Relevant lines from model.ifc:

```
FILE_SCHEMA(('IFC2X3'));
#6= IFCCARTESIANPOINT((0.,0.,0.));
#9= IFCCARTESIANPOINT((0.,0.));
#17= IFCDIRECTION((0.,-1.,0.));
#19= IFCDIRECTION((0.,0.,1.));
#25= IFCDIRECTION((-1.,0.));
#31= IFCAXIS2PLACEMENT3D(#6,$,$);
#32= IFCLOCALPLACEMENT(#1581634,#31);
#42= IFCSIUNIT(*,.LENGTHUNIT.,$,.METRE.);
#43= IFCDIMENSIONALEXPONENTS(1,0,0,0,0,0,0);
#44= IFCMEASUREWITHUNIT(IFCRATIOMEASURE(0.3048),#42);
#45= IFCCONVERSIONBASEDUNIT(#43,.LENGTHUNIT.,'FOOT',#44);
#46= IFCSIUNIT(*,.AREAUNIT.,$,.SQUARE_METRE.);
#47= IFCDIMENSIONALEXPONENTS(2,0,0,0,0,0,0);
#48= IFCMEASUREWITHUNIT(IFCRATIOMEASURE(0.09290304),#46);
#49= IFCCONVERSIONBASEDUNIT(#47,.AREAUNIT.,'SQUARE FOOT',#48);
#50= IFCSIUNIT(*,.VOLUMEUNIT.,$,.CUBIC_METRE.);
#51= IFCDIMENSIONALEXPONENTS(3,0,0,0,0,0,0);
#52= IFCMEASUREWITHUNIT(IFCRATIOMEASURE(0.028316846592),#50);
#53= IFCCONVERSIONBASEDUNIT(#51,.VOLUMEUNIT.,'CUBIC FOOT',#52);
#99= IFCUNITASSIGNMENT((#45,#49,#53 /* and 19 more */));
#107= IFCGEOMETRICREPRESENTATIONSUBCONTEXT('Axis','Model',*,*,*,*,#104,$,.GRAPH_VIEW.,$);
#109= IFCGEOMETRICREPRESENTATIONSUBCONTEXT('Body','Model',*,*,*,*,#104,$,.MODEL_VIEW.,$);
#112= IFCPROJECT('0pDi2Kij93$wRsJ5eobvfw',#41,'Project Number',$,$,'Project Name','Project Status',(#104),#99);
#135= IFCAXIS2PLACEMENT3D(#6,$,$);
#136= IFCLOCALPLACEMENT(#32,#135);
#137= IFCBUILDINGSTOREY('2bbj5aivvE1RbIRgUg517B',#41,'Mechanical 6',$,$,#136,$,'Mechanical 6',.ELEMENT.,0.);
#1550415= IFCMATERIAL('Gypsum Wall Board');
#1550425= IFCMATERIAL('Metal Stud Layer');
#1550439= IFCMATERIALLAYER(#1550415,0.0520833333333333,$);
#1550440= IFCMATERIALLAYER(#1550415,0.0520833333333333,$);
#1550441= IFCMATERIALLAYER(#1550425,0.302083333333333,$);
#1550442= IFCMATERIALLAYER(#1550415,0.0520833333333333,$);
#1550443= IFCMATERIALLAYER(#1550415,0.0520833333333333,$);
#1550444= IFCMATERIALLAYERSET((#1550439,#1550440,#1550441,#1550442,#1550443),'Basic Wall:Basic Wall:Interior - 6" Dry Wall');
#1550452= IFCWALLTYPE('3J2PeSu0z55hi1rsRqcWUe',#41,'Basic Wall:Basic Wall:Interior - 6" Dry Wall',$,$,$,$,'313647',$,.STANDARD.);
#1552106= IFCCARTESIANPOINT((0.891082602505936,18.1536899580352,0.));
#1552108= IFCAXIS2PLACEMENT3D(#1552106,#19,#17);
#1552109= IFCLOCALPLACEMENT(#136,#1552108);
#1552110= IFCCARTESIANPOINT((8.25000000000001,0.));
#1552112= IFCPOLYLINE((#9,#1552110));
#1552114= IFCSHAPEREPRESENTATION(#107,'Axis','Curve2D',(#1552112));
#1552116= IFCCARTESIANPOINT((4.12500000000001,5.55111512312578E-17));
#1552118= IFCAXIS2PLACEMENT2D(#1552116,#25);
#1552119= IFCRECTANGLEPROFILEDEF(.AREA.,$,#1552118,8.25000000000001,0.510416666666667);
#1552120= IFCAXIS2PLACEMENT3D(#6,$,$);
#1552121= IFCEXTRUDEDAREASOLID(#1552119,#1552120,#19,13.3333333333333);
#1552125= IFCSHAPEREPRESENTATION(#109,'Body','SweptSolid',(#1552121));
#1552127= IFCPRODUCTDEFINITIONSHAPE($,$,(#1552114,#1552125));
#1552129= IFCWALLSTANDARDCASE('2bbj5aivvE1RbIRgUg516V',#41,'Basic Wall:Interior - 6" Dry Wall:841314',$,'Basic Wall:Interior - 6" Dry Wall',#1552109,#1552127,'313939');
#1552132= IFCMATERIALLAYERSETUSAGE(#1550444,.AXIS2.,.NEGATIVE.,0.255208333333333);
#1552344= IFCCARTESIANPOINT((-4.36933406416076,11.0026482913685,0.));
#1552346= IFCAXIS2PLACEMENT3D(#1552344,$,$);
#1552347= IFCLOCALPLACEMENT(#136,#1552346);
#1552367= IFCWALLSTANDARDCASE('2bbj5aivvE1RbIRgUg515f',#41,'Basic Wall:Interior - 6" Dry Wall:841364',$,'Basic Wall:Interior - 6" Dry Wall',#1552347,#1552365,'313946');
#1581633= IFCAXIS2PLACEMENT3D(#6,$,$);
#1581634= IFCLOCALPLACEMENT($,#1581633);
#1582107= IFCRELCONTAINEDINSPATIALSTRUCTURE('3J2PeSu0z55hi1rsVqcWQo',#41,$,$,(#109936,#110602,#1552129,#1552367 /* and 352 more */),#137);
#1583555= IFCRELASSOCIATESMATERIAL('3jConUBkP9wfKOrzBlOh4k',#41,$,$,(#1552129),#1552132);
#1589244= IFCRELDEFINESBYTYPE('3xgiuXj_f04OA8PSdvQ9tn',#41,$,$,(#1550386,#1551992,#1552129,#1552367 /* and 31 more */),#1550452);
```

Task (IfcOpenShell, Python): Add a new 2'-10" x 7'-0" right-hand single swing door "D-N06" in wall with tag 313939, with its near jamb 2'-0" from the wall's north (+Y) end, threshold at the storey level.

```python
import numpy as np
import ifcopenshell
import ifcopenshell.api.feature
import ifcopenshell.api.geometry
import ifcopenshell.api.root
import ifcopenshell.api.spatial
import ifcopenshell.api.type
import ifcopenshell.geom
import ifcopenshell.util.element
import ifcopenshell.util.placement
import ifcopenshell.util.representation
import ifcopenshell.util.shape
import ifcopenshell.util.unit

model = ifcopenshell.open("model.ifc")
unit_scale = ifcopenshell.util.unit.calculate_unit_scale(model)
settings = ifcopenshell.geom.settings()


def volume(element):
    """Net volume in cubic metres, openings subtracted."""
    shape = ifcopenshell.geom.create_shape(settings, element)
    return ifcopenshell.util.shape.get_volume(shape.geometry)


wall = model.by_guid("2bbj5aivvE1RbIRgUg516V")
storey = ifcopenshell.util.element.get_container(wall, ifc_class="IfcBuildingStorey")
context = ifcopenshell.util.representation.get_context(model, "Model", "Body", "MODEL_VIEW")
before = volume(wall)

width, height, from_end, sill = 0.8636, 2.1336, 0.6096, 0.0  # metres

# The wall runs along its own X axis, and the end named is its -X end.
wall_shape = ifcopenshell.geom.create_shape(settings, wall)
x, y, z = ifcopenshell.util.shape.get_vertices(wall_shape.geometry).T
start = x.min() + from_end
face, thickness = float(y.min()), float(y.max() - y.min())
wall_matrix = ifcopenshell.util.placement.get_local_placement(wall.ObjectPlacement)
level = ifcopenshell.util.placement.get_local_placement(storey.ObjectPlacement)[2, 3]


def in_wall(x, y):
    """Placement at x, y metres in the wall's axes, at sill height."""
    matrix = wall_matrix.copy()
    matrix[:, 3] = wall_matrix @ np.array([x / unit_scale, y / unit_scale, 0.0, 1.0])
    matrix[2, 3] = level + sill / unit_scale
    return matrix


# Opening: a box that overshoots both wall faces by 50 mm.
opening = ifcopenshell.api.root.create_entity(model, ifc_class="IfcOpeningElement")
box = ifcopenshell.api.geometry.add_wall_representation(
    model, context=context, length=width, height=height, thickness=thickness + 0.1
)
ifcopenshell.api.geometry.assign_representation(model, product=opening, representation=box)
ifcopenshell.api.geometry.edit_object_placement(model, product=opening, matrix=in_wall(start, face - 0.05), is_si=False)
ifcopenshell.api.feature.add_feature(model, feature=opening, element=wall)

door = ifcopenshell.api.root.create_entity(model, ifc_class="IfcDoor", name="D-N06")
door.OverallWidth, door.OverallHeight = width / unit_scale, height / unit_scale
body = ifcopenshell.api.geometry.add_door_representation(
    model,
    context=context,
    overall_width=door.OverallWidth,
    overall_height=door.OverallHeight,
    operation_type="SINGLE_SWING_RIGHT",
    lining_properties={"LiningDepth": thickness / unit_scale, "ThresholdDepth": thickness / unit_scale},
)
ifcopenshell.api.geometry.assign_representation(model, product=door, representation=body)
ifcopenshell.api.spatial.assign_container(model, products=[door], relating_structure=storey)
fills = ifcopenshell.api.feature.add_filling(model, opening=opening, element=door)
fills.OwnerHistory = door.OwnerHistory  # required in IFC2X3

# IFC2X3 keeps the operation on the door style.
style = ifcopenshell.api.root.create_entity(model, ifc_class="IfcDoorStyle", name="D-N06")
style.OperationType, style.ConstructionType = "SINGLE_SWING_RIGHT", "NOTDEFINED"
style.ParameterTakesPrecedence = style.Sizeable = False
ifcopenshell.api.type.assign_type(model, related_objects=[door], relating_type=style)

# The lining spans the wall, so the door starts at the wall face.
ifcopenshell.api.geometry.edit_object_placement(model, product=door, matrix=in_wall(start, face), is_si=False)

after = volume(wall)

print(f"wall volume {before:.3f} -> {after:.3f} m3")

model.write("model_rev.ifc")
```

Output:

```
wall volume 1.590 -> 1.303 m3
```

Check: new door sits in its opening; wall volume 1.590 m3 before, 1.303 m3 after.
